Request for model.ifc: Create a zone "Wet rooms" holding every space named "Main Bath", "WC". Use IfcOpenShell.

First a look at what the model holds.

```python
import ifcopenshell

model = ifcopenshell.open("model.ifc")
print(model.schema)
seen = {}
for space in model.by_type("IfcSpace"):
    seen[space.LongName] = seen.get(space.LongName, 0) + 1
for name, count in sorted(seen.items(), key=str):
    print(count, "x", name)
print("zones:", [z.Name for z in model.by_type("IfcZone")][:20])
```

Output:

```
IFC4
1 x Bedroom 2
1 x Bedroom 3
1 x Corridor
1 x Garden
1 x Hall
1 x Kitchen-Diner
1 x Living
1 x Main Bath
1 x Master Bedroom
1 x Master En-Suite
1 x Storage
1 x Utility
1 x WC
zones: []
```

```python
import ifcopenshell
import ifcopenshell.api.group
import ifcopenshell.api.root

model = ifcopenshell.open("model.ifc")

names = {"Main Bath", "WC"}
spaces = [s for s in model.by_type("IfcSpace") if s.LongName in names]

zone = ifcopenshell.api.root.create_entity(model, ifc_class="IfcZone", name="Wet rooms")
ifcopenshell.api.group.assign_group(model, products=spaces, group=zone)
print(len(spaces), "spaces in", zone.Name)

model.write("model_updated.ifc")
```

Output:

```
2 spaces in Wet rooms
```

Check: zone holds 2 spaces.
